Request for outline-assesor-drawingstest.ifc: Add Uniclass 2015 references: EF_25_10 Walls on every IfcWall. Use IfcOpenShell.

First a look at what the model holds.

```python
import ifcopenshell

model = ifcopenshell.open("outline-assesor-drawingstest.ifc")
print(model.schema)
print("classifications:", [c.Name for c in model.by_type("IfcClassification")])
for ifc_class in ("IfcDoor", "IfcRoof", "IfcStair", "IfcWall", "IfcWindow"):
    print(ifc_class, len(model.by_type(ifc_class)))
```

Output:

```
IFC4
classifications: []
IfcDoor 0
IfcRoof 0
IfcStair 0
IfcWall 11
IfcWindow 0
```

```python
import ifcopenshell
import ifcopenshell.api.classification

model = ifcopenshell.open("outline-assesor-drawingstest.ifc")

system = ifcopenshell.api.classification.add_classification(model, classification="Uniclass 2015")

codes = {
    "IfcWall": ("EF_25_10", "Walls"),
}
for ifc_class, (code, name) in codes.items():
    products = model.by_type(ifc_class)
    ifcopenshell.api.classification.add_reference(
        model, products=products, classification=system, identification=code, name=name
    )
    print(code, len(products))

model.write("outline-assesor-drawingstest-out.ifc")
```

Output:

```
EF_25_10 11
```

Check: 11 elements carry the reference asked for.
